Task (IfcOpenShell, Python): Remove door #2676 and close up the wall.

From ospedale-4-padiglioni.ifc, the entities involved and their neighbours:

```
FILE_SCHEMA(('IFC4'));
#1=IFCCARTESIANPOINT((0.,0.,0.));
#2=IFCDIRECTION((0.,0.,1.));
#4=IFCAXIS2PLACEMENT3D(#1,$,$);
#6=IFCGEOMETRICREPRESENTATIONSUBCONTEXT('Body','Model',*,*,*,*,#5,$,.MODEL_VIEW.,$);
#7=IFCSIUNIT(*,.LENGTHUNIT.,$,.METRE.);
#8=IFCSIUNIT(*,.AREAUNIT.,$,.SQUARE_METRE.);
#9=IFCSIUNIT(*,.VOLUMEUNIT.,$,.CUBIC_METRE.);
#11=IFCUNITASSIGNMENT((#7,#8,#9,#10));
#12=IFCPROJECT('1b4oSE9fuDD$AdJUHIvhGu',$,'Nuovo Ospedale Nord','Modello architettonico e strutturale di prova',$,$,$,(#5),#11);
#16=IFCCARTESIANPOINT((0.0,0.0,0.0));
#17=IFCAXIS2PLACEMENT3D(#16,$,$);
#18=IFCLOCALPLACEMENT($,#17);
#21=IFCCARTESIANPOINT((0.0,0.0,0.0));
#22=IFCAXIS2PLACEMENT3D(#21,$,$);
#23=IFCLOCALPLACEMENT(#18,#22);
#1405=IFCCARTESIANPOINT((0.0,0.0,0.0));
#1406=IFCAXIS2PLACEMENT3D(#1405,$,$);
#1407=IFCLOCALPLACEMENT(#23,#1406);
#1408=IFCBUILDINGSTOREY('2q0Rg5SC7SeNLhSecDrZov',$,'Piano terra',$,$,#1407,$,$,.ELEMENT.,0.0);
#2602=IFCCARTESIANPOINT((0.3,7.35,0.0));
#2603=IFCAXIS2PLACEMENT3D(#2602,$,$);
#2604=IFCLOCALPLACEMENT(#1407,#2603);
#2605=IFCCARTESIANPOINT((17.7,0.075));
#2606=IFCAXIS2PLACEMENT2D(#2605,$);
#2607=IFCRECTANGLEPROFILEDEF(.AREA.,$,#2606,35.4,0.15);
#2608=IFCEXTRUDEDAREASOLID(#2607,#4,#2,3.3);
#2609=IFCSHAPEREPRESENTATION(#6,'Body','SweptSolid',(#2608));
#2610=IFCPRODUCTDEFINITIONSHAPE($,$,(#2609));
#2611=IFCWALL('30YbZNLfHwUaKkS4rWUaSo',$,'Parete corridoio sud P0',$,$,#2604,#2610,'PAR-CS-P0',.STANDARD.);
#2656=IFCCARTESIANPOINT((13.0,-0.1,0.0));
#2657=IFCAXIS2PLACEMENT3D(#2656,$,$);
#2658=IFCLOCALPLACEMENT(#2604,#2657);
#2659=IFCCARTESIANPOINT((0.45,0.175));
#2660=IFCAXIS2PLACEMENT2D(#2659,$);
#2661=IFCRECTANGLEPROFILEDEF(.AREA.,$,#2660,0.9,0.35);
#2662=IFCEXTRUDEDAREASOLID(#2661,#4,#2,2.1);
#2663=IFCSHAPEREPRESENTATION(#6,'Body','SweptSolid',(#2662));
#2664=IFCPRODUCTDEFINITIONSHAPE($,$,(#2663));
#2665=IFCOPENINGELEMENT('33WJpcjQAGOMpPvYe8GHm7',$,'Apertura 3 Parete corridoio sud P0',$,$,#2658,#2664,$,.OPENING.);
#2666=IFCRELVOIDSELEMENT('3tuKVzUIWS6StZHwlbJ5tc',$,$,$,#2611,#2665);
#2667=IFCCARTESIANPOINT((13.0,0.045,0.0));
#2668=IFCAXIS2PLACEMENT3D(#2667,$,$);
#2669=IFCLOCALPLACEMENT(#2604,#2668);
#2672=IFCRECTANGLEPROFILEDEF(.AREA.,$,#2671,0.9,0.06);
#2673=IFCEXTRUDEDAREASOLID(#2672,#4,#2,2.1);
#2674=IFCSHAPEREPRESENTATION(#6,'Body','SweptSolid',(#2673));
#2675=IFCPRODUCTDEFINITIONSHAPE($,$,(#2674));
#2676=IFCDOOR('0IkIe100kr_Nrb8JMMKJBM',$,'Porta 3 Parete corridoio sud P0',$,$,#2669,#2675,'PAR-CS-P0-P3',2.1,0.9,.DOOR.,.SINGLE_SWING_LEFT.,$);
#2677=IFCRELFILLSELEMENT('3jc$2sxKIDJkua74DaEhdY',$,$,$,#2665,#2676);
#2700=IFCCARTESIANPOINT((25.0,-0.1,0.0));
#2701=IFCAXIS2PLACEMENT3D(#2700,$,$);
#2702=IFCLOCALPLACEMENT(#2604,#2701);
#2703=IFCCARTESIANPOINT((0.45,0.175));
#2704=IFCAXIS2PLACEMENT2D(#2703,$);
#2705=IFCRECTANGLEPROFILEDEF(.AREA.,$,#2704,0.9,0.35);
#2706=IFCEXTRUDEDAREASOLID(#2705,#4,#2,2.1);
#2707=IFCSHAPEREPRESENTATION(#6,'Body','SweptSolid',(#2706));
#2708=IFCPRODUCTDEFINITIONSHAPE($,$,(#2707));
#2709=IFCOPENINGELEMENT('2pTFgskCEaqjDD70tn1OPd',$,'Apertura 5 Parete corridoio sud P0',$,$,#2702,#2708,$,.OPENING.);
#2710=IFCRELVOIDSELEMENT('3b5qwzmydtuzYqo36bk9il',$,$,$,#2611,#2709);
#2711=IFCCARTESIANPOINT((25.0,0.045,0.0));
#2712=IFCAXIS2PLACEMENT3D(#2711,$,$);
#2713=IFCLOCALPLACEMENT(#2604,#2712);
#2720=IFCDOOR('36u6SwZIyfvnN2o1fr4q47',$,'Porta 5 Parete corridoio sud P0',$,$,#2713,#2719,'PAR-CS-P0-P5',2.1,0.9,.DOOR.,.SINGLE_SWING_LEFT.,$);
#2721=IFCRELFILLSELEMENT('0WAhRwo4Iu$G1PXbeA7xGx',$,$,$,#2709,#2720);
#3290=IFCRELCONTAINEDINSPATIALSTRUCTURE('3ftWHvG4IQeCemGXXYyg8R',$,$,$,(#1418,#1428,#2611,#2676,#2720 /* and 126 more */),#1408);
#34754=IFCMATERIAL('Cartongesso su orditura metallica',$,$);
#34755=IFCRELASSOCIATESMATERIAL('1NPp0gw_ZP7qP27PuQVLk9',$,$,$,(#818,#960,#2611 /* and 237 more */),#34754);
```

```python
import ifcopenshell
import ifcopenshell.api.feature
import ifcopenshell.api.root
import ifcopenshell.geom
import ifcopenshell.util.shape

model = ifcopenshell.open("ospedale-4-padiglioni.ifc")
settings = ifcopenshell.geom.settings()


def volume(element):
    """Net volume in cubic metres, openings subtracted."""
    shape = ifcopenshell.geom.create_shape(settings, element)
    return ifcopenshell.util.shape.get_volume(shape.geometry)


door = model.by_guid("0IkIe100kr_Nrb8JMMKJBM")
opening = door.FillsVoids[0].RelatingOpeningElement
wall = opening.VoidsElements[0].RelatingBuildingElement
before = volume(wall)

ifcopenshell.api.root.remove_product(model, product=door)
ifcopenshell.api.feature.remove_feature(model, feature=opening)

after = volume(wall)

print(f"wall volume {before:.3f} -> {after:.3f} m3")

model.write("ospedale-4-padiglioni-out.ifc")
```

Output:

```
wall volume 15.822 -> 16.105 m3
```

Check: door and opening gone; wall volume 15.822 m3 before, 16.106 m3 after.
